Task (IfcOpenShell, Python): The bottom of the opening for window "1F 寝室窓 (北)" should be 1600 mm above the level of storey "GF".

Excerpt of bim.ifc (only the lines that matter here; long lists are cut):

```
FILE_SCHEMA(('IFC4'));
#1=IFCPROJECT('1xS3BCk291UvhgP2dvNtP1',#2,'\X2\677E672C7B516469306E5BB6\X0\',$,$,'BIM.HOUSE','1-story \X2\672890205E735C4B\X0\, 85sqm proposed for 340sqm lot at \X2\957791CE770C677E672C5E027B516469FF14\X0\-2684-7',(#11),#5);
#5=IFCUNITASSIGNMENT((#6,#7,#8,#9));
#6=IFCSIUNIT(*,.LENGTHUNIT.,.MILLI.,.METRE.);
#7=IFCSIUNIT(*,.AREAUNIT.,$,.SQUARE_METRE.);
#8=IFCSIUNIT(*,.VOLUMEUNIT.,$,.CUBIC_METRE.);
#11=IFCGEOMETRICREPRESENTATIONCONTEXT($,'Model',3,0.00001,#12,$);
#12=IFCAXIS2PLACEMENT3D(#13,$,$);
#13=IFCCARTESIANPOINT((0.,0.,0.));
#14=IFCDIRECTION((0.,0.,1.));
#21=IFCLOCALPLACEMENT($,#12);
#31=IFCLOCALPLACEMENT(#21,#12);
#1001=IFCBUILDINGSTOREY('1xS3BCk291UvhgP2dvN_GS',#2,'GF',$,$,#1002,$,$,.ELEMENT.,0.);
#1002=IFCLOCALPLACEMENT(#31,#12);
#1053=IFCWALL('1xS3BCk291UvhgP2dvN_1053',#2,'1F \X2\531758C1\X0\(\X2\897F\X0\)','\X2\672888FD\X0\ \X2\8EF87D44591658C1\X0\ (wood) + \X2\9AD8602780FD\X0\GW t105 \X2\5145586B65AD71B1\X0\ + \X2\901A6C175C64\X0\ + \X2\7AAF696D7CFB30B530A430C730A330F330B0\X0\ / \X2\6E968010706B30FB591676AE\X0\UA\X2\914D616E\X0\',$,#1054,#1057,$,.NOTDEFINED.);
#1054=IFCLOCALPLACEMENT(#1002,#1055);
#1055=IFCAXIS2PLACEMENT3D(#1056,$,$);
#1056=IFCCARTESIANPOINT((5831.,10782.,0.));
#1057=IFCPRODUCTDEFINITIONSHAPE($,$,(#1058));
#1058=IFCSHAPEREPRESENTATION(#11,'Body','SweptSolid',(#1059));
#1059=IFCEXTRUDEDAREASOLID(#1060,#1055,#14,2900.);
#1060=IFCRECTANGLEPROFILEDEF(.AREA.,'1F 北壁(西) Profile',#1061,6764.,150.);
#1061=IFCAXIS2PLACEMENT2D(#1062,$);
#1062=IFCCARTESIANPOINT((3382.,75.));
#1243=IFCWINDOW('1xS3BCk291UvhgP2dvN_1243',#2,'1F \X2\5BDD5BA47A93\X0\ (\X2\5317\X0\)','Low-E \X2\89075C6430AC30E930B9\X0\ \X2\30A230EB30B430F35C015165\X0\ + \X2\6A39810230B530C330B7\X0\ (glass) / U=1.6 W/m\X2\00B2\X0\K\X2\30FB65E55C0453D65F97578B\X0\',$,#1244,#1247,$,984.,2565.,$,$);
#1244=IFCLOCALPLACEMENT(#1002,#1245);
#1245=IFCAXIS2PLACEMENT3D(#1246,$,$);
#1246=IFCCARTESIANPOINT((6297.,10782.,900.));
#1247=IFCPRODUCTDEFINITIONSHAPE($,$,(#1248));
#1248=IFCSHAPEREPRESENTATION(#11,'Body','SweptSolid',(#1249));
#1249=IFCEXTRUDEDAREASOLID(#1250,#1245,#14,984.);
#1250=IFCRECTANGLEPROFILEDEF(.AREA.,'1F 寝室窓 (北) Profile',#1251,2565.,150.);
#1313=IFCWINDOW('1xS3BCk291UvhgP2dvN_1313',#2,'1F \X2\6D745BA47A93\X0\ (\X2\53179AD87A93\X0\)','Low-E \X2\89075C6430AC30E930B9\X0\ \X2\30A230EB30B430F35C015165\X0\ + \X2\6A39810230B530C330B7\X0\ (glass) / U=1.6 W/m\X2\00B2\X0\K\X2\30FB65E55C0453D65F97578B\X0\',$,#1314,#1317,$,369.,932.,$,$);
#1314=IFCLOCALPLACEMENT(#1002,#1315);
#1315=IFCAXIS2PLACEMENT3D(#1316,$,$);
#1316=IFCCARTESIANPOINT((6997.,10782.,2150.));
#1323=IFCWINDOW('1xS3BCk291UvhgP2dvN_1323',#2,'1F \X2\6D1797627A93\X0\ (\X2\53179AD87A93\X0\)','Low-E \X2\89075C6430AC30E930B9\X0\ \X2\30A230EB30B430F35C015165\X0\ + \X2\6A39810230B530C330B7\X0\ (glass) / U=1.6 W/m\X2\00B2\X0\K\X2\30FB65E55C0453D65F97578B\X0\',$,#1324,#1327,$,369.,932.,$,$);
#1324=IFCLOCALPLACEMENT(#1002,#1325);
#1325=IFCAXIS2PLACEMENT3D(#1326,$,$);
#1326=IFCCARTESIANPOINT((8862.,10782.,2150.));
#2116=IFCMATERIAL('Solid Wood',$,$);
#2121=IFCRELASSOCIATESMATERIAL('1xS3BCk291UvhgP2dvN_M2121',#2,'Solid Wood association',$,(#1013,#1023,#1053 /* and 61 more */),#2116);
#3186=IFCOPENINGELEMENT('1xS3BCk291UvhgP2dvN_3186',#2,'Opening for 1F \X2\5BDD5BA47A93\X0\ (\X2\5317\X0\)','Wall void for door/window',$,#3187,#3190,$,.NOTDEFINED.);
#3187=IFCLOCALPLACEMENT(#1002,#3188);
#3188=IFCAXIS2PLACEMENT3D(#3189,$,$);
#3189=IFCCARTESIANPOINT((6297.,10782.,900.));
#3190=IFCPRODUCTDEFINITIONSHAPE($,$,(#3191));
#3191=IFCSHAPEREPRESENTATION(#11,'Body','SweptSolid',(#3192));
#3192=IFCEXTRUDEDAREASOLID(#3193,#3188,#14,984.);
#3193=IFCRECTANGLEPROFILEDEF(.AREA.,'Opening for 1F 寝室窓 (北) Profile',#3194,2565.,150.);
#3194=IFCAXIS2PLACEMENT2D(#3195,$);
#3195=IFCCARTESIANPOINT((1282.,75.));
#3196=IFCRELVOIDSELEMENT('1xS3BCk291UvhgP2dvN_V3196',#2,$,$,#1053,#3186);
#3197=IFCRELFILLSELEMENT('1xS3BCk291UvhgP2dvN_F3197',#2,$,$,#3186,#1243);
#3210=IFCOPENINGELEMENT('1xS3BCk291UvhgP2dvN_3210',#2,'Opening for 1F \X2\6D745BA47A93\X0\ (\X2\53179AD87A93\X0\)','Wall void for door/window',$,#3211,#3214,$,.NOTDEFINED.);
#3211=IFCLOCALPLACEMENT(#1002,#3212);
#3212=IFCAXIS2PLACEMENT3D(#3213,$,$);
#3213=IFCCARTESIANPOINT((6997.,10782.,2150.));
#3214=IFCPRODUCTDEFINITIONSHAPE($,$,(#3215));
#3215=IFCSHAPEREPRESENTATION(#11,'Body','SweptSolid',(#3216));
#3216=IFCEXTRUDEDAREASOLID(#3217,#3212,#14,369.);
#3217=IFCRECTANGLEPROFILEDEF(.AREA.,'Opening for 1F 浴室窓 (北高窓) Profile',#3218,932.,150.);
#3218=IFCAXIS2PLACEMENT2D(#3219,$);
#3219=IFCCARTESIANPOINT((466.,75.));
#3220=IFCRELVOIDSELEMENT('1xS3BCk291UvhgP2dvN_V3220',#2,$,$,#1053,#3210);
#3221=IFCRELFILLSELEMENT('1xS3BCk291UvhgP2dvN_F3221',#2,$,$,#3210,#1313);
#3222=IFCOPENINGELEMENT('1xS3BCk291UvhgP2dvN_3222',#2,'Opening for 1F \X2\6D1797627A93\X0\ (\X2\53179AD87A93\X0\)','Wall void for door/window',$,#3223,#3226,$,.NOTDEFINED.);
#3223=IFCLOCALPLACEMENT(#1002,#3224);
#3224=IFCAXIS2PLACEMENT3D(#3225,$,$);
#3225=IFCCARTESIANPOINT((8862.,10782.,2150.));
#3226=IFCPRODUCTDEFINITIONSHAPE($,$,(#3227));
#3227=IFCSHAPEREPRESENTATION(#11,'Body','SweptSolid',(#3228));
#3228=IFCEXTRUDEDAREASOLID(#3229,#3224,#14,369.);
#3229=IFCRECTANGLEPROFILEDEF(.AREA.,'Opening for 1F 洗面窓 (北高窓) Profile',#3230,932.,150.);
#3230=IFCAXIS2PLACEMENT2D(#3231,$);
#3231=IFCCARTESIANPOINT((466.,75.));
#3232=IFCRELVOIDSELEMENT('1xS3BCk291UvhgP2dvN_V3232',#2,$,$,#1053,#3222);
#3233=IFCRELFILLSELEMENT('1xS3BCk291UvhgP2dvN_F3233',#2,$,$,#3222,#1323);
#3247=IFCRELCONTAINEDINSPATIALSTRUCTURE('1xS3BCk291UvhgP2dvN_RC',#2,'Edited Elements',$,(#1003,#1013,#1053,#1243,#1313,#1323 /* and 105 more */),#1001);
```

```python
import numpy as np
import ifcopenshell
import ifcopenshell.api.geometry
import ifcopenshell.geom
import ifcopenshell.util.element
import ifcopenshell.util.placement
import ifcopenshell.util.shape
import ifcopenshell.util.unit

model = ifcopenshell.open("bim.ifc")
unit_scale = ifcopenshell.util.unit.calculate_unit_scale(model)

window = model.by_guid("1xS3BCk291UvhgP2dvN_1243")
opening = window.FillsVoids[0].RelatingOpeningElement
storey = ifcopenshell.util.element.get_container(window, ifc_class="IfcBuildingStorey")
level = ifcopenshell.util.placement.get_local_placement(storey.ObjectPlacement)[2, 3]

# The opening's origin need not be at the sill, so measure its lowest point.
shape = ifcopenshell.geom.create_shape(ifcopenshell.geom.settings(), opening)
bottom = ifcopenshell.util.shape.get_shape_bottom_elevation(shape, shape.geometry) / unit_scale
dz = level + 1600.0 - bottom

shift = np.array([0.0, 0.0, dz])
# The window is not placed relative to its opening, so move both.
for product in (opening, window):
    matrix = ifcopenshell.util.placement.get_local_placement(product.ObjectPlacement)
    matrix[:3, 3] += shift
    ifcopenshell.api.geometry.edit_object_placement(model, product=product, matrix=matrix, is_si=False)

print(f"moved by {dz * unit_scale:+.3f} m")

model.write("bim_updated.ifc")
```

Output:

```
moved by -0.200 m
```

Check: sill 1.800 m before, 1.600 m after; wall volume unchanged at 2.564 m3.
